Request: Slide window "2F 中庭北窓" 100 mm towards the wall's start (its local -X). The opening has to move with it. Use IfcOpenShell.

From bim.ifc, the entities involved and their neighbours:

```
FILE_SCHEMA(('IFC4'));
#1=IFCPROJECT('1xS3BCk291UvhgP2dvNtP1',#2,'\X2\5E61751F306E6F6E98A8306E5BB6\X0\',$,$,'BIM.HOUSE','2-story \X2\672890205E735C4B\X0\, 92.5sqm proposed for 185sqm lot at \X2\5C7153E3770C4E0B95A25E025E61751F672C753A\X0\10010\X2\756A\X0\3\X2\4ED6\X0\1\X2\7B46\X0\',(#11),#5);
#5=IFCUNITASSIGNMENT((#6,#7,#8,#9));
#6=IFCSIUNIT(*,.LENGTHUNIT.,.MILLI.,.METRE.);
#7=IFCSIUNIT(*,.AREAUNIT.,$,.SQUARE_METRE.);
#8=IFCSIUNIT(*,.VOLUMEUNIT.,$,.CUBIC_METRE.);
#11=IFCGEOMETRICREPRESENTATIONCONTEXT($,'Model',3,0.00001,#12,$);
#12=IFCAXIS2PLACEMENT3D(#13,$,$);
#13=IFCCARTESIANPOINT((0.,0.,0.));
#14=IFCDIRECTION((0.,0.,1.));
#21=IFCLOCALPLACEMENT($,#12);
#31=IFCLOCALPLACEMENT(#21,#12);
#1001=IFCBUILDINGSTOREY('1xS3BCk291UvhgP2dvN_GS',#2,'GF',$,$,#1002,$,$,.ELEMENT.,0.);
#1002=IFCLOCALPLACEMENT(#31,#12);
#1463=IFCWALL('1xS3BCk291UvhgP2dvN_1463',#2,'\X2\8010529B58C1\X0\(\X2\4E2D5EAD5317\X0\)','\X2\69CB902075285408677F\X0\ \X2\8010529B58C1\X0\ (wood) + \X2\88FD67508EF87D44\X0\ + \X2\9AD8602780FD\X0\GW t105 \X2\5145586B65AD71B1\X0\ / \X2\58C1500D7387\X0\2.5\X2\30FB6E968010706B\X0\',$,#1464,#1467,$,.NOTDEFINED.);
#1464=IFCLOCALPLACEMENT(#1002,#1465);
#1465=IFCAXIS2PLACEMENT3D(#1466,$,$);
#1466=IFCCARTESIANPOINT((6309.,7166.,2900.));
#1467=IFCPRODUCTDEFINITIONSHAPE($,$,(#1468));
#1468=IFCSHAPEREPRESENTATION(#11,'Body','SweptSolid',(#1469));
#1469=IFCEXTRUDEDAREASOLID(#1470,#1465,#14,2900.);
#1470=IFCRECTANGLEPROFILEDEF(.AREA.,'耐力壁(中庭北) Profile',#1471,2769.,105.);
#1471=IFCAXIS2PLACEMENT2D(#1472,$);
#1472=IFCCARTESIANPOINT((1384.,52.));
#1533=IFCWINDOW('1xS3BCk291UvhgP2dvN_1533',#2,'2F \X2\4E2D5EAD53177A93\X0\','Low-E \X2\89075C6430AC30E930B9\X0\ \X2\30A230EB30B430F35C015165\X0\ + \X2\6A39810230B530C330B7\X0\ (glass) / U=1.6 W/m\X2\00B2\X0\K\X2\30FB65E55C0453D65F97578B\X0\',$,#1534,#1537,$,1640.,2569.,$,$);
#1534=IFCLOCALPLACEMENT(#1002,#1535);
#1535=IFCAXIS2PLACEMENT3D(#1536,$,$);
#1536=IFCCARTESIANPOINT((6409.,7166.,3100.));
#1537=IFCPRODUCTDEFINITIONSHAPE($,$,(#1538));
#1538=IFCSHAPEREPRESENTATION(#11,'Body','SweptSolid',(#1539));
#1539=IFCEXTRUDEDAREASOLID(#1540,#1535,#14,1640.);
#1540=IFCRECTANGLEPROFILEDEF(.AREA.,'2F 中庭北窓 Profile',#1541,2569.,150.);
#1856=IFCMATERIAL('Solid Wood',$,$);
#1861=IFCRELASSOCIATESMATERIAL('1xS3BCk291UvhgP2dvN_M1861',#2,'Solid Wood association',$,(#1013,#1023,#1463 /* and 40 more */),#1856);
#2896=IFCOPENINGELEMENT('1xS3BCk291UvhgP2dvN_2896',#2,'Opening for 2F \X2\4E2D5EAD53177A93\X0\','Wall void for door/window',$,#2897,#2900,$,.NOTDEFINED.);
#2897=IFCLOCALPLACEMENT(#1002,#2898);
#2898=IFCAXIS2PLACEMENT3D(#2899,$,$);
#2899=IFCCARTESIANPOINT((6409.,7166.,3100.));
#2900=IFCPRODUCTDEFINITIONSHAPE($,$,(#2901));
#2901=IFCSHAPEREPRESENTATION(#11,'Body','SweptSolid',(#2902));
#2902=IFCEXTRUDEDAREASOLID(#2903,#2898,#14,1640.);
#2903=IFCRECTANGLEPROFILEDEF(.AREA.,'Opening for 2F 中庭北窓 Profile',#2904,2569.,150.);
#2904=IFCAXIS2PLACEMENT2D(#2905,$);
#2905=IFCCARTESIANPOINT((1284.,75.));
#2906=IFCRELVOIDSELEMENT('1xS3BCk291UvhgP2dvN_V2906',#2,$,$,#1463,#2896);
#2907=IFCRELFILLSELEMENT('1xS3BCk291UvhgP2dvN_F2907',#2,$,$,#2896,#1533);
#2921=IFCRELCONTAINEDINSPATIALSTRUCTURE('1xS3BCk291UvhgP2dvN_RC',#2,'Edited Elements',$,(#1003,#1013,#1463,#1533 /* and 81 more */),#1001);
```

```python
import ifcopenshell
import ifcopenshell.api.geometry
import ifcopenshell.util.placement
import ifcopenshell.util.unit

model = ifcopenshell.open("bim.ifc")
unit_scale = ifcopenshell.util.unit.calculate_unit_scale(model)

window = model.by_id(1533)
opening = window.FillsVoids[0].RelatingOpeningElement
wall = opening.VoidsElements[0].RelatingBuildingElement

wall_matrix = ifcopenshell.util.placement.get_local_placement(wall.ObjectPlacement)
shift = wall_matrix[:3, 0] * -0.1 / unit_scale
before = ifcopenshell.util.placement.get_local_placement(window.ObjectPlacement)[:3, 3].copy()

# The window is not placed relative to its opening, so move both.
for product in (opening, window):
    matrix = ifcopenshell.util.placement.get_local_placement(product.ObjectPlacement)
    matrix[:3, 3] += shift
    ifcopenshell.api.geometry.edit_object_placement(model, product=product, matrix=matrix, is_si=False)

after = ifcopenshell.util.placement.get_local_placement(window.ObjectPlacement)[:3, 3]
print("window moved by", (after - before).round(3) + 0.0)

model.write("bim_rev.ifc")
```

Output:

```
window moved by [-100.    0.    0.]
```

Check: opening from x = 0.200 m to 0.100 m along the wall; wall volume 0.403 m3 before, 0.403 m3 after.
